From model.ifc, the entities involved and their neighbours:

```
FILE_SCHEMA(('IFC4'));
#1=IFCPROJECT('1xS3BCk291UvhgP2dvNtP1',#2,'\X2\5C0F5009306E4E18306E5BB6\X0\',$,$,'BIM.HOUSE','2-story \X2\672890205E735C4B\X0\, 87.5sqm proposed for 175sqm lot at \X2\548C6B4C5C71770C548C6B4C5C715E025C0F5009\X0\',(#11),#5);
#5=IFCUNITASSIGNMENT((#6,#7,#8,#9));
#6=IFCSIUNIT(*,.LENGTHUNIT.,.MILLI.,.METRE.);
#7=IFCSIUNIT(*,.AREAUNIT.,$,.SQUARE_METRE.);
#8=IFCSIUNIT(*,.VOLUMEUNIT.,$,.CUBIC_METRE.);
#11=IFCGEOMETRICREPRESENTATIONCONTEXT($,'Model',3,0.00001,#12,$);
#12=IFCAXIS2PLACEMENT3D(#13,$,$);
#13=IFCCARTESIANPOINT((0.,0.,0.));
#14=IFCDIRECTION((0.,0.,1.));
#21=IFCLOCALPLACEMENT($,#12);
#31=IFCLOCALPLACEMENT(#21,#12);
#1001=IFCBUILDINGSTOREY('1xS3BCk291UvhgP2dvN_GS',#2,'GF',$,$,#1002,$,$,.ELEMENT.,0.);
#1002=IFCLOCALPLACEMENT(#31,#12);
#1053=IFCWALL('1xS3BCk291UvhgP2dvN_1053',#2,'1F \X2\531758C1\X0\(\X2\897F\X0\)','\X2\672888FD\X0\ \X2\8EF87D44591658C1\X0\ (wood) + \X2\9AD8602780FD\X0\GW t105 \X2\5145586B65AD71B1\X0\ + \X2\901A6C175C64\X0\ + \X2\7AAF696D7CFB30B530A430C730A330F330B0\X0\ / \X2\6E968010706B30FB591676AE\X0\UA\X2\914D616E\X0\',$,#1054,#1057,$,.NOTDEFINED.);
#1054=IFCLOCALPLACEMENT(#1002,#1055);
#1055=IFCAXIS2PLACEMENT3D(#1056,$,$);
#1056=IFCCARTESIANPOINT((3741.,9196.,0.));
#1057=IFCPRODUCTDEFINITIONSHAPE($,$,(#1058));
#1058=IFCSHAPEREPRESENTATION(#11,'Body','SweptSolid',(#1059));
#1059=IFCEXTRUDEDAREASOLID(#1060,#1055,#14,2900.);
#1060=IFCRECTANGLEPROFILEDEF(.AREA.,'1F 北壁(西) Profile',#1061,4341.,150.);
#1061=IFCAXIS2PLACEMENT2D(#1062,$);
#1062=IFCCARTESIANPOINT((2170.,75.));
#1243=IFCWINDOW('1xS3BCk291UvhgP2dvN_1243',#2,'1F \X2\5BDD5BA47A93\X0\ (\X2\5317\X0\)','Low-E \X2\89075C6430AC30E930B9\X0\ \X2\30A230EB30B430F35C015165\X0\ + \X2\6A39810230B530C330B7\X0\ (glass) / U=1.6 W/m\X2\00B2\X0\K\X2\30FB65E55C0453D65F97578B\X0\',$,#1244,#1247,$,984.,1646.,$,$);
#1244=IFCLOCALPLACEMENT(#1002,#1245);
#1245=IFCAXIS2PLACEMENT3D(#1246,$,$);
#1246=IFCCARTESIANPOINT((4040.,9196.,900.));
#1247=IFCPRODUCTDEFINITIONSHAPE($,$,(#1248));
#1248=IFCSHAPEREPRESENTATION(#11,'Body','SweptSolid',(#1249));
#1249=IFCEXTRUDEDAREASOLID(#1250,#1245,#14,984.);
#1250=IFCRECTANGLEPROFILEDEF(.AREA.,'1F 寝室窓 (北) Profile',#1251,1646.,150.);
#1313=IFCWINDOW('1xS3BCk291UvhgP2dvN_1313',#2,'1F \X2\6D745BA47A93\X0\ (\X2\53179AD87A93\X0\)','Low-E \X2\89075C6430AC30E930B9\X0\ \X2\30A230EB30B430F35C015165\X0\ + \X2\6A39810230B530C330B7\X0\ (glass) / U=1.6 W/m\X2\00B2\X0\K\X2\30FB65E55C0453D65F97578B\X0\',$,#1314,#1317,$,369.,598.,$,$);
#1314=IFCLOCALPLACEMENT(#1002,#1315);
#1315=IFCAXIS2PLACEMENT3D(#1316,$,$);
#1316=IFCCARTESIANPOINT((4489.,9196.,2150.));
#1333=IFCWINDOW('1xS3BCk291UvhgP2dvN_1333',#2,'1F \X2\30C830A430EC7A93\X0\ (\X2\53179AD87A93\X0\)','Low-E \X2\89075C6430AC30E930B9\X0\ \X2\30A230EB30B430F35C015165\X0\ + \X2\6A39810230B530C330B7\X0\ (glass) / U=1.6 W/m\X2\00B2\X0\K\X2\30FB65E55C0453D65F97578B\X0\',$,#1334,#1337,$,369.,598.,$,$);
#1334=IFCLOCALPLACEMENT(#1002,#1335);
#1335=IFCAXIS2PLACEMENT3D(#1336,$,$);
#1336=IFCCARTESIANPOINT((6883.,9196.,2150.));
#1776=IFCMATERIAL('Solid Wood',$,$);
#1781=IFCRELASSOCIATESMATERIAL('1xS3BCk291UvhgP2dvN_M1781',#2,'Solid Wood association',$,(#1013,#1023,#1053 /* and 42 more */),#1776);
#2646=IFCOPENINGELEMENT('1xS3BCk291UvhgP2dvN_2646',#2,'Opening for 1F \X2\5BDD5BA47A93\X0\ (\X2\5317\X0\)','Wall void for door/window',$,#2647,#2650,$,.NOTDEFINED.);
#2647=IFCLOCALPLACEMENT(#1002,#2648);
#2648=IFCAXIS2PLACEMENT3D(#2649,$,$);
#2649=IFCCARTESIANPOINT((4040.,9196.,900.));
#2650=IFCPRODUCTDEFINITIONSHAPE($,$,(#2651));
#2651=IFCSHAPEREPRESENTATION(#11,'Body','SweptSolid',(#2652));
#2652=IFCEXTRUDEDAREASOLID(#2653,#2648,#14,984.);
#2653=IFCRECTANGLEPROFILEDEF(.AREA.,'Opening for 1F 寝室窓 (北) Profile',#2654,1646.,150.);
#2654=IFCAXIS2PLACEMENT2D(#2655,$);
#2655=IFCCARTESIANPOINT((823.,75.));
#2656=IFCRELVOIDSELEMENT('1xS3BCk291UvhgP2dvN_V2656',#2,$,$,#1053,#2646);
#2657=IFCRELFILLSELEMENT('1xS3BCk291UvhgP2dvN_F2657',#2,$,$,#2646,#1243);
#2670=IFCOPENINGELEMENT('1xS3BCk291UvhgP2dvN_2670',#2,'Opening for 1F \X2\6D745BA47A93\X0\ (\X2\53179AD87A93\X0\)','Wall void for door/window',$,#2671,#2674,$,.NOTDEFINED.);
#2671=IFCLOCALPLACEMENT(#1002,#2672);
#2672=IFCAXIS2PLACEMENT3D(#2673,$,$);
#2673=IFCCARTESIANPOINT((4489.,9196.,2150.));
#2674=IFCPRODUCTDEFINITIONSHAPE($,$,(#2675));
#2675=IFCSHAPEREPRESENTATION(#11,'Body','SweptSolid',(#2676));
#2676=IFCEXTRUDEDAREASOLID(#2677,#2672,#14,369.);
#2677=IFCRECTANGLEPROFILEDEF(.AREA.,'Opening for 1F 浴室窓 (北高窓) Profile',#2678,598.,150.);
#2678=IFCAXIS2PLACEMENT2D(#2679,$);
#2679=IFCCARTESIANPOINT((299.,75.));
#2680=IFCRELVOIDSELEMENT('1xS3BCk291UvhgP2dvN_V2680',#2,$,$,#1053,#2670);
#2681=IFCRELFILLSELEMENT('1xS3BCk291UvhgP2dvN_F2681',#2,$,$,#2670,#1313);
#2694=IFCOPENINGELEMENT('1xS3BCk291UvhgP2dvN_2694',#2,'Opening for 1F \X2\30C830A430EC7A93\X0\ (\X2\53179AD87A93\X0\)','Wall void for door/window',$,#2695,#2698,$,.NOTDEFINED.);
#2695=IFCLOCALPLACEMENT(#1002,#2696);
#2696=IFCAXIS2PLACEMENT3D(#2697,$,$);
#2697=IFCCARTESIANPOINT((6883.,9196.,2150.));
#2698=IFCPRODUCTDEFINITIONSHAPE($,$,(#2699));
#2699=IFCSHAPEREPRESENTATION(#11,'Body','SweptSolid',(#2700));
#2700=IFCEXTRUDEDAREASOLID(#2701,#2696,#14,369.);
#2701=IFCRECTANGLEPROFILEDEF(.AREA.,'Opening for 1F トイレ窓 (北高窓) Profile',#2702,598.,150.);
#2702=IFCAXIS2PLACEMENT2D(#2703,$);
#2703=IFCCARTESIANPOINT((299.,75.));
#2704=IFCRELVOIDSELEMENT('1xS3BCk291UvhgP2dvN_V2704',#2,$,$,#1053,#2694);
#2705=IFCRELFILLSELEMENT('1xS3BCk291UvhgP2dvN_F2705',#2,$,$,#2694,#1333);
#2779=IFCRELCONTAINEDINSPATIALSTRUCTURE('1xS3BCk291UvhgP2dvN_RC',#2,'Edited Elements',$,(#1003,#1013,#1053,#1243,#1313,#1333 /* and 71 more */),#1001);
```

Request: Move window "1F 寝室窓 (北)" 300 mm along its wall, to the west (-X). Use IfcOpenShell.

```python
import ifcopenshell
import ifcopenshell.api.geometry
import ifcopenshell.util.placement
import ifcopenshell.util.unit

model = ifcopenshell.open("model.ifc")
unit_scale = ifcopenshell.util.unit.calculate_unit_scale(model)

window = model.by_guid("1xS3BCk291UvhgP2dvN_1243")
opening = window.FillsVoids[0].RelatingOpeningElement
wall = opening.VoidsElements[0].RelatingBuildingElement

wall_matrix = ifcopenshell.util.placement.get_local_placement(wall.ObjectPlacement)
shift = wall_matrix[:3, 0] * -0.3 / unit_scale
before = ifcopenshell.util.placement.get_local_placement(window.ObjectPlacement)[:3, 3].copy()

# The window is not placed relative to its opening, so move both.
for product in (opening, window):
    matrix = ifcopenshell.util.placement.get_local_placement(product.ObjectPlacement)
    matrix[:3, 3] += shift
    ifcopenshell.api.geometry.edit_object_placement(model, product=product, matrix=matrix, is_si=False)

after = ifcopenshell.util.placement.get_local_placement(window.ObjectPlacement)[:3, 3]
print("window moved by", (after - before).round(3) + 0.0)

model.write("model_v2.ifc")
```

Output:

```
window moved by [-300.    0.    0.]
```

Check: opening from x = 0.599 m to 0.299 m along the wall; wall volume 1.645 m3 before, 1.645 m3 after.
